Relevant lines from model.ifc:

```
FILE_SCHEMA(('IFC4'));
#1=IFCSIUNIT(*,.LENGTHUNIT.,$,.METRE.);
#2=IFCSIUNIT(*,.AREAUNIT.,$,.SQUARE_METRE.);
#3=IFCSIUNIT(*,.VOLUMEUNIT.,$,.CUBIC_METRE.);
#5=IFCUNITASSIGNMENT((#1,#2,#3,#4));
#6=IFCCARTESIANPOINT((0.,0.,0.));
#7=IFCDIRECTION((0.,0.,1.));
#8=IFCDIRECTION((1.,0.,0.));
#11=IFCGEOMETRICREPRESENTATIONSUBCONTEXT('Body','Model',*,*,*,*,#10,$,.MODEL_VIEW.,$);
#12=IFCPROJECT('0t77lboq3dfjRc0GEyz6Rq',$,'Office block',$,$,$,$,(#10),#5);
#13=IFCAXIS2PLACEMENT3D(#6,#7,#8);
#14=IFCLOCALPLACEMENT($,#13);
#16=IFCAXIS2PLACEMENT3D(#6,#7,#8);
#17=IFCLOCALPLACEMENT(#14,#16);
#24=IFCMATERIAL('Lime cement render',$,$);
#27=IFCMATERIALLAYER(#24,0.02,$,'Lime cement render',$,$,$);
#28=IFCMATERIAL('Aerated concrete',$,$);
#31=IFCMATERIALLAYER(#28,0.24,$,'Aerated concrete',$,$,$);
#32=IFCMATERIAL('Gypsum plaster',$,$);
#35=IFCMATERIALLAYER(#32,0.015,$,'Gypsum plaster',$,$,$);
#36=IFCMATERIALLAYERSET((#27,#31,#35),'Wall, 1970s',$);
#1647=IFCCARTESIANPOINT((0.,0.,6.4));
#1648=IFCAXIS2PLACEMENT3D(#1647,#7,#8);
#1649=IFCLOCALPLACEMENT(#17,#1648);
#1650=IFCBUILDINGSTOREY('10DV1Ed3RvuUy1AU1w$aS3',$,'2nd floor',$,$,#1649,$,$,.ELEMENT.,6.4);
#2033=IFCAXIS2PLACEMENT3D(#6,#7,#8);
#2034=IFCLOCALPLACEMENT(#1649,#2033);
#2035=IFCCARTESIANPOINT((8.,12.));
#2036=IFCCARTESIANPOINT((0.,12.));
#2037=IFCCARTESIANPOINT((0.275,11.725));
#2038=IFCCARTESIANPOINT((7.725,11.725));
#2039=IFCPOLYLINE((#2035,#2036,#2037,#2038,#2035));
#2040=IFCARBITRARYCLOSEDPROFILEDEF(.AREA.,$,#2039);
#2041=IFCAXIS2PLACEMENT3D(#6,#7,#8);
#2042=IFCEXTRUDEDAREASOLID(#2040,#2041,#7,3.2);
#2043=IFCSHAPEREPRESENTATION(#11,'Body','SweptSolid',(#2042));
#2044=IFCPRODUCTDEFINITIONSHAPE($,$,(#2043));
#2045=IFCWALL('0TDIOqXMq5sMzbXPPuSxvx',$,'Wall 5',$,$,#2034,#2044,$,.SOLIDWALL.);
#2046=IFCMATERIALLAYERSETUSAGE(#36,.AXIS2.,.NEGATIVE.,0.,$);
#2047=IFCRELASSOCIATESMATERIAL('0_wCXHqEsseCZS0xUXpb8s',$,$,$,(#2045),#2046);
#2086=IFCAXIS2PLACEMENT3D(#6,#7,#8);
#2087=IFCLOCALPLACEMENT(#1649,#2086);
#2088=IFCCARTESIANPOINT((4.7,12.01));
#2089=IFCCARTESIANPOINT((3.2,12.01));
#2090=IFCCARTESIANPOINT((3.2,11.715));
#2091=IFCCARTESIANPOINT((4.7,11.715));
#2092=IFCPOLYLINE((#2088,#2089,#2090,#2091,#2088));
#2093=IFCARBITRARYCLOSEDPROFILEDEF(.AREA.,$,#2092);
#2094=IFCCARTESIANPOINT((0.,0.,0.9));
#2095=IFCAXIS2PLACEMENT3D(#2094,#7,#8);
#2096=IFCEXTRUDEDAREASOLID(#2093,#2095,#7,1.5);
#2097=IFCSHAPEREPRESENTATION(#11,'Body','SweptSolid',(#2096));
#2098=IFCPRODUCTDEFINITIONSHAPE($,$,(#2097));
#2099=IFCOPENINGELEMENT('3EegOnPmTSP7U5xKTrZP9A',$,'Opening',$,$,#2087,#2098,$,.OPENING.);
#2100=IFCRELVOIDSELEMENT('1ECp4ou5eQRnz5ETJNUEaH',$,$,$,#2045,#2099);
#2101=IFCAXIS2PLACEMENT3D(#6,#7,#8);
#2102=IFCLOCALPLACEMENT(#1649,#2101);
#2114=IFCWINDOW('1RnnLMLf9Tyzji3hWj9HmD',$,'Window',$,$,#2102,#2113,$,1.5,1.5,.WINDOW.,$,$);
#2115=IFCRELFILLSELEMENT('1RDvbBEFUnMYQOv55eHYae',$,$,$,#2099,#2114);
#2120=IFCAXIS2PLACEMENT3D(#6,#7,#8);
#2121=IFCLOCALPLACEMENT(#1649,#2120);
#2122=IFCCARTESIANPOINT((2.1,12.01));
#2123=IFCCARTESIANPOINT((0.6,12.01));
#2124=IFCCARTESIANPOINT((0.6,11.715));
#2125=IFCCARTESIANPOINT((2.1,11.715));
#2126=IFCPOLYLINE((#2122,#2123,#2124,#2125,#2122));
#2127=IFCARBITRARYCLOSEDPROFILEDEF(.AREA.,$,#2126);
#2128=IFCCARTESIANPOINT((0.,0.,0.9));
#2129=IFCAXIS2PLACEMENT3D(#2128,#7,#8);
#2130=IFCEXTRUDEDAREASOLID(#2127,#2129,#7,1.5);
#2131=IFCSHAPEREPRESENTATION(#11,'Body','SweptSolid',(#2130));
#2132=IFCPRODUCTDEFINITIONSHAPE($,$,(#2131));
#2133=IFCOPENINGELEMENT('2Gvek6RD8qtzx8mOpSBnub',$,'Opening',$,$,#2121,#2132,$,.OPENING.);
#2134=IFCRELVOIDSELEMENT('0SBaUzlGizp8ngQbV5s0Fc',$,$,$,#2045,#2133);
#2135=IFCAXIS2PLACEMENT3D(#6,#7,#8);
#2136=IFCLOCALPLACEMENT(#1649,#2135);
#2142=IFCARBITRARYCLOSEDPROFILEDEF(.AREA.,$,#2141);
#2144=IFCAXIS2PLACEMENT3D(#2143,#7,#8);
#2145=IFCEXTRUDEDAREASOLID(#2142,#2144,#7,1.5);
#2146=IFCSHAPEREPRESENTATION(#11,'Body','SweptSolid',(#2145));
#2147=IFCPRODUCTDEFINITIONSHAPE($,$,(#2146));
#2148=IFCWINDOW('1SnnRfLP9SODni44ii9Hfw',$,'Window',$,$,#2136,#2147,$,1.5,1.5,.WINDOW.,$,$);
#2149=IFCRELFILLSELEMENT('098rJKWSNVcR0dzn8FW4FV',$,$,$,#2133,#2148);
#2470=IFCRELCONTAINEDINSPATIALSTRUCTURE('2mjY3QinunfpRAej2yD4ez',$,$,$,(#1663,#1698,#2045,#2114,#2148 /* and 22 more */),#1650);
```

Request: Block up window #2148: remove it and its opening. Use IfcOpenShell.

```python
import ifcopenshell
import ifcopenshell.api.feature
import ifcopenshell.api.root
import ifcopenshell.geom
import ifcopenshell.util.shape

model = ifcopenshell.open("model.ifc")
settings = ifcopenshell.geom.settings()


def volume(element):
    """Net volume in cubic metres, openings subtracted."""
    shape = ifcopenshell.geom.create_shape(settings, element)
    return ifcopenshell.util.shape.get_volume(shape.geometry)


window = model.by_guid("1SnnRfLP9SODni44ii9Hfw")
opening = window.FillsVoids[0].RelatingOpeningElement
wall = opening.VoidsElements[0].RelatingBuildingElement
before = volume(wall)

ifcopenshell.api.root.remove_product(model, product=window)
ifcopenshell.api.feature.remove_feature(model, feature=opening)

after = volume(wall)

print(f"wall volume {before:.3f} -> {after:.3f} m3")

model.write("model-out.ifc")
```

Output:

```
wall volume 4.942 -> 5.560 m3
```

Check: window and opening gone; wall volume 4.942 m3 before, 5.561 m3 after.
